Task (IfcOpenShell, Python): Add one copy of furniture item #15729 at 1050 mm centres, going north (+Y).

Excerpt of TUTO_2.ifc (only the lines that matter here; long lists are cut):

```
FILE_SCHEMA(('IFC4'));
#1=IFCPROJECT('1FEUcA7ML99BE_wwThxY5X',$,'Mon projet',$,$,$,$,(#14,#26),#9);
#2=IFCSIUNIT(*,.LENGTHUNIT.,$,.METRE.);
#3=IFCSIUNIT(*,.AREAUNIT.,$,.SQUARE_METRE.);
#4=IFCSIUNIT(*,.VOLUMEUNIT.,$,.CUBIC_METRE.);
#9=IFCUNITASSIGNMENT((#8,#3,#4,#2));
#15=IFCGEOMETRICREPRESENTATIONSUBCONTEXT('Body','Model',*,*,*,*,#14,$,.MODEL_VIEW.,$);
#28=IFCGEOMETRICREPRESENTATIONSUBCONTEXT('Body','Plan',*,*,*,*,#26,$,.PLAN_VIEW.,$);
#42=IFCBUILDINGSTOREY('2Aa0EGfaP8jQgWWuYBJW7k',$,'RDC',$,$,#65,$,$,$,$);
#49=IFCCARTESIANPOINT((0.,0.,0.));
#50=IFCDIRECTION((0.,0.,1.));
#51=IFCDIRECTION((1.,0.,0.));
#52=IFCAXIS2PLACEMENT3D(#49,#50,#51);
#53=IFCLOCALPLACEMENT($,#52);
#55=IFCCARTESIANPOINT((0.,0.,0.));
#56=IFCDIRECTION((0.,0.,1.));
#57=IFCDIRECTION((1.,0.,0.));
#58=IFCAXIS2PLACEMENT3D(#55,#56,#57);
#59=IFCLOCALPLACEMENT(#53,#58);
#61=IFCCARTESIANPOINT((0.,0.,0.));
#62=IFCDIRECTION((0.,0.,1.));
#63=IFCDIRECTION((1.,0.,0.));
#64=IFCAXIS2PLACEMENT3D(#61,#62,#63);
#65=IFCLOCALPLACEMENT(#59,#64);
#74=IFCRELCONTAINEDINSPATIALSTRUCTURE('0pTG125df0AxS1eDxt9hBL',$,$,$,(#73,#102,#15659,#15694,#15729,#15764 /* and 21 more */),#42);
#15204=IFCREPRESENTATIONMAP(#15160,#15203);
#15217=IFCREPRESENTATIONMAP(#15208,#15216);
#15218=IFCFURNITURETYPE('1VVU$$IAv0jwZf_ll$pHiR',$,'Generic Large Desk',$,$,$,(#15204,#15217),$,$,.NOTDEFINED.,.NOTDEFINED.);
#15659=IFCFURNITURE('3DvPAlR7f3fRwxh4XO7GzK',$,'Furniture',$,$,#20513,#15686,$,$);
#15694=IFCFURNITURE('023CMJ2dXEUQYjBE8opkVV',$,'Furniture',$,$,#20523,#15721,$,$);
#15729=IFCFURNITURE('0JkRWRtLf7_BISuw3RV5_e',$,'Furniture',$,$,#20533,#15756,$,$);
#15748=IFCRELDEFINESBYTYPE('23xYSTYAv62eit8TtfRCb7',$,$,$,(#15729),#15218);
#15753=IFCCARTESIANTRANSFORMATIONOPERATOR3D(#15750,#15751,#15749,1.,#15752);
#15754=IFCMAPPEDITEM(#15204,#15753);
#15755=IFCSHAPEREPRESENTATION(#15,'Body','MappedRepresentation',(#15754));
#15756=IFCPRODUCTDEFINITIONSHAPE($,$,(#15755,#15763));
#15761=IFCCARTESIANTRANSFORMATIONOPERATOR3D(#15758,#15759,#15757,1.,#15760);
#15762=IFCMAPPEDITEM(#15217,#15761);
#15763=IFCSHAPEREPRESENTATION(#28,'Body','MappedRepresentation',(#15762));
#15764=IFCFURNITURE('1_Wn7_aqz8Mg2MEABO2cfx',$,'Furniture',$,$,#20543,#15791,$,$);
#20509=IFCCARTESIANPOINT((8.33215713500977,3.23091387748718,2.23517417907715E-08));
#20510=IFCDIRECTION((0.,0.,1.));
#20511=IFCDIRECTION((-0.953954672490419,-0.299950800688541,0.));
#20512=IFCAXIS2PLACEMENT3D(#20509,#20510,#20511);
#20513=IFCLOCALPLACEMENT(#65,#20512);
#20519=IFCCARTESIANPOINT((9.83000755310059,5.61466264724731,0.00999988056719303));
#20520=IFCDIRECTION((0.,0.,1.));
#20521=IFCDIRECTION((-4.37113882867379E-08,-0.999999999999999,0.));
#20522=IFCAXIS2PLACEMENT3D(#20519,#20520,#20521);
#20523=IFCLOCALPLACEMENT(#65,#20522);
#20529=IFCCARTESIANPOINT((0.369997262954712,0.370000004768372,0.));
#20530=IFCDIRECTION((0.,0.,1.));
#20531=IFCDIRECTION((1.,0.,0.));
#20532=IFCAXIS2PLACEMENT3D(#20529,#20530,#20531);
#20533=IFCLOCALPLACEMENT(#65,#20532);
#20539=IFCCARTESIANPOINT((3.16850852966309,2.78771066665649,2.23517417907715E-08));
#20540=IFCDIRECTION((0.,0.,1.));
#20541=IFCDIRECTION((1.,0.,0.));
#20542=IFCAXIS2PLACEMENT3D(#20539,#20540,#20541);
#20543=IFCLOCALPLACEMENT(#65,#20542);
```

```python
import numpy as np
import ifcopenshell
import ifcopenshell.api.geometry
import ifcopenshell.api.root
import ifcopenshell.util.element
import ifcopenshell.util.placement
import ifcopenshell.util.unit

model = ifcopenshell.open("TUTO_2.ifc")
unit_scale = ifcopenshell.util.unit.calculate_unit_scale(model)

source = model.by_id(15729)
base = ifcopenshell.util.placement.get_local_placement(source.ObjectPlacement)
step = np.array([0.0, 1.0, 0.0]) * 1.05 / unit_scale

for i in range(1, 2):
    copy = ifcopenshell.api.root.copy_class(model, product=source)
    copy.Representation = ifcopenshell.util.element.copy_deep(
        model, source.Representation, exclude=["IfcGeometricRepresentationContext", "IfcRepresentationMap"]
    )
    matrix = base.copy()
    matrix[:3, 3] += i * step
    print("added at", matrix[:3, 3].round(3) + 0.0)
    ifcopenshell.api.geometry.edit_object_placement(model, product=copy, matrix=matrix, is_si=False)

model.write("TUTO_2-out.ifc")
```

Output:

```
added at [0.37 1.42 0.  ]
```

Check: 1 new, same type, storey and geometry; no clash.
